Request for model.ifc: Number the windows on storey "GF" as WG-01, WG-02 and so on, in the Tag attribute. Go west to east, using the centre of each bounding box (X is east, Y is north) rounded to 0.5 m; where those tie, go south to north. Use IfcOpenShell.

First a look at what the model holds.

```python
import ifcopenshell
import ifcopenshell.util.element
import ifcopenshell.util.placement

model = ifcopenshell.open("model.ifc")
print(model.schema)
storey = next(s for s in model.by_type("IfcBuildingStorey") if s.Name == "GF")
windows = [e for e in ifcopenshell.util.element.get_decomposition(storey) if e.is_a("IfcWindow")]
for e in sorted(windows, key=lambda e: e.id()):
    origin = ifcopenshell.util.placement.get_local_placement(e.ObjectPlacement)[:3, 3]
    print(e.id(), e.Tag, e.Name, origin.round(2) + 0.0, sep=" | ")
```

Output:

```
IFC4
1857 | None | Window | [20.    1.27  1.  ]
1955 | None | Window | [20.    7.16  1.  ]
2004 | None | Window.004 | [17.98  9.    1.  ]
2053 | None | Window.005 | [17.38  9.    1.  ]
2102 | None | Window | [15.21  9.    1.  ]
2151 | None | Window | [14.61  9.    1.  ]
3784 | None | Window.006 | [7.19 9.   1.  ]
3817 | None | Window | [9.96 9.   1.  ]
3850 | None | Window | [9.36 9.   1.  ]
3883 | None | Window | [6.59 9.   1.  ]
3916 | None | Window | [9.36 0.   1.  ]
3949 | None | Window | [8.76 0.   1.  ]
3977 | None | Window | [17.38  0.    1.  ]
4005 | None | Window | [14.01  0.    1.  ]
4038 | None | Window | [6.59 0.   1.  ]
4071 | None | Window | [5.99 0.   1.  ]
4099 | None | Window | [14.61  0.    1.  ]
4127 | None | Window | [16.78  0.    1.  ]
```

```python
import ifcopenshell
import ifcopenshell.geom
import ifcopenshell.util.element
import ifcopenshell.util.shape

model = ifcopenshell.open("model.ifc")
settings = ifcopenshell.geom.settings()
settings.set("use-world-coords", True)


def centre(element):
    shape = ifcopenshell.geom.create_shape(settings, element)
    return ifcopenshell.util.shape.get_bbox_centroid(shape.geometry)


storey = next(s for s in model.by_type("IfcBuildingStorey") if s.Name == "GF")
windows = [e for e in ifcopenshell.util.element.get_decomposition(storey) if e.is_a("IfcWindow")]

# Insertion points can sit at a corner or the storey origin, so sort by the geometry (in metres).
centres = {e: centre(e) for e in windows}
windows.sort(key=lambda e: (round(centres[e][0] / 0.5), centres[e][1]))

for i, e in enumerate(windows, start=1):
    number = f"WG-{i:02d}"
    e.Tag = number
    print(e.id(), number)

model.write("model_rev.ifc")
```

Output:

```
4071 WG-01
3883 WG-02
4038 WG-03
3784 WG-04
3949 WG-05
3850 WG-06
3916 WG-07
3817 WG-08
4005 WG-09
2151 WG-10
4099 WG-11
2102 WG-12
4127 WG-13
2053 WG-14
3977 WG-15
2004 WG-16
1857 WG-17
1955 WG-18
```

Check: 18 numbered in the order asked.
